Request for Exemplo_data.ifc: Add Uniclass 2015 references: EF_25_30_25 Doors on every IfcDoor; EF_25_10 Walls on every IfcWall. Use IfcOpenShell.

First a look at what the model holds.

```python
import ifcopenshell

model = ifcopenshell.open("Exemplo_data.ifc")
print(model.schema)
print("classifications:", [c.Name for c in model.by_type("IfcClassification")])
for ifc_class in ("IfcDoor", "IfcRoof", "IfcStair", "IfcWall", "IfcWindow"):
    print(ifc_class, len(model.by_type(ifc_class)))
```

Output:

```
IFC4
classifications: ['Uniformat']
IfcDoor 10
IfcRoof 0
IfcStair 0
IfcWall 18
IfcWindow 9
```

```python
import ifcopenshell
import ifcopenshell.api.classification

model = ifcopenshell.open("Exemplo_data.ifc")

system = ifcopenshell.api.classification.add_classification(model, classification="Uniclass 2015")

codes = {
    "IfcDoor": ("EF_25_30_25", "Doors"),
    "IfcWall": ("EF_25_10", "Walls"),
}
for ifc_class, (code, name) in codes.items():
    products = model.by_type(ifc_class)
    ifcopenshell.api.classification.add_reference(
        model, products=products, classification=system, identification=code, name=name
    )
    print(code, len(products))

model.write("Exemplo_data-out.ifc")
```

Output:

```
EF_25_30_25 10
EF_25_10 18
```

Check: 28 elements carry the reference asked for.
